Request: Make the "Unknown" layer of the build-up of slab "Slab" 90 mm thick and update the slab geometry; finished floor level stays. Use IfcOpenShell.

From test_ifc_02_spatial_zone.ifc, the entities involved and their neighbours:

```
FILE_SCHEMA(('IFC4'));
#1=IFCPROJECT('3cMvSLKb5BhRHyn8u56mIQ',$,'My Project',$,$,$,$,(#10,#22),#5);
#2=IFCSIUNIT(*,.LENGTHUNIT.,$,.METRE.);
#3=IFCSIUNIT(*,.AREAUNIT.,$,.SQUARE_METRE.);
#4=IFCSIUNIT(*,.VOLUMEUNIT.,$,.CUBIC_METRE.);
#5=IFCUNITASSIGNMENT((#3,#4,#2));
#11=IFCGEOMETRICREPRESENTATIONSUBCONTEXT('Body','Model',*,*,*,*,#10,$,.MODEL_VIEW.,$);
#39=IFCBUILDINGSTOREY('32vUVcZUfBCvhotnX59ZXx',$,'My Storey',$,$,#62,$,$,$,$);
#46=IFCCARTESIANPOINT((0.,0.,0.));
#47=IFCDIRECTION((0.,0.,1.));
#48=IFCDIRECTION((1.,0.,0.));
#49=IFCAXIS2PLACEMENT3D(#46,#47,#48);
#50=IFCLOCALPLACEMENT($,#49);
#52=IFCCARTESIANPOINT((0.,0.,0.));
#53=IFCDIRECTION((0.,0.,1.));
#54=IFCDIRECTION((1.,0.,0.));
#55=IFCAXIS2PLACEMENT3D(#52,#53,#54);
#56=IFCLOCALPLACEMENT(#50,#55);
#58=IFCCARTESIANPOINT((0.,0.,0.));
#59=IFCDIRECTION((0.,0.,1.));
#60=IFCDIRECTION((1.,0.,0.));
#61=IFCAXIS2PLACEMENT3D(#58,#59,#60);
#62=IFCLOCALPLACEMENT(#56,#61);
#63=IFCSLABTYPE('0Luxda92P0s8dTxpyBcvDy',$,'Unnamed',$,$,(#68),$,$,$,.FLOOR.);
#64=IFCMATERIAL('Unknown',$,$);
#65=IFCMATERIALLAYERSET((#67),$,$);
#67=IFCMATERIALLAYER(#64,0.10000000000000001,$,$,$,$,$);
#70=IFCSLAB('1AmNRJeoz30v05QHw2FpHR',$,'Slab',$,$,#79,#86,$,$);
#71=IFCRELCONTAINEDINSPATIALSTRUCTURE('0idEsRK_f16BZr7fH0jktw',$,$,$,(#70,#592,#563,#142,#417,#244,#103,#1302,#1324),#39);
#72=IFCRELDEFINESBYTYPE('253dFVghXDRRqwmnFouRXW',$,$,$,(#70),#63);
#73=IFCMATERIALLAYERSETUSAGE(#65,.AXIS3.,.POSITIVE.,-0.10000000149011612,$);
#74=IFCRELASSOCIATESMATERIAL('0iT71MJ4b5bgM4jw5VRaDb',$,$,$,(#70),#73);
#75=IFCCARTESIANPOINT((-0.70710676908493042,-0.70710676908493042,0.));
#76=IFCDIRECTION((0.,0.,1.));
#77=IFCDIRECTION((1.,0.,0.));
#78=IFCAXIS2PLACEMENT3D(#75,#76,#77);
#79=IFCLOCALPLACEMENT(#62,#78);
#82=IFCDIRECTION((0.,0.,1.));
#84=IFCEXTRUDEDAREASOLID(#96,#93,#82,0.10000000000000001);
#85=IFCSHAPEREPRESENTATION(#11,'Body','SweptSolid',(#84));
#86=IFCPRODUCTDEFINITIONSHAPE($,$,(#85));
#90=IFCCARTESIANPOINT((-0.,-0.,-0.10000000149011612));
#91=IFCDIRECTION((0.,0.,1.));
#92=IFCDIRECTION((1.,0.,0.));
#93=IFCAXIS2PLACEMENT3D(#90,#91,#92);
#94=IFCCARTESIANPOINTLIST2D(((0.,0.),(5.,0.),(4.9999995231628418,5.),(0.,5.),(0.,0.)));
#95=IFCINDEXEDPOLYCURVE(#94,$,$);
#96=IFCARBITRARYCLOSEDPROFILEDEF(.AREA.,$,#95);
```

```python
import ifcopenshell
import ifcopenshell.util.element
import ifcopenshell.util.representation
import ifcopenshell.util.unit

model = ifcopenshell.open("test_ifc_02_spatial_zone.ifc")
unit_scale = ifcopenshell.util.unit.calculate_unit_scale(model)

layer_set = model.by_id(65)
layer = next(l for l in layer_set.MaterialLayers if l.Material and l.Material.Name == "Unknown")
change = 0.09 / unit_scale - layer.LayerThickness
layer.LayerThickness += change

# Geometry does not follow the layer set by itself.
slabs = [e for e in ifcopenshell.util.element.get_elements_by_material(model, layer_set) if e.is_a("IfcSlab")]
for slab in sorted(slabs, key=lambda e: e.id()):
    body = ifcopenshell.util.representation.get_representation(slab, "Model", "Body")
    solid = body.Items[0]
    old_depth = solid.Depth
    solid.Depth += change
    # Extruded upwards: lower the start of the extrusion so the top stays.
    x, y, z = solid.Position.Location.Coordinates
    solid.Position.Location = model.createIfcCartesianPoint((x, y, z - change))
    print(slab.id(), f"{old_depth:g} -> {solid.Depth:g}")

# The layers are counted up from the underside, which has moved.
for usage in {ifcopenshell.util.element.get_material(slab) for slab in slabs}:
    usage.OffsetFromReferenceLine -= change

model.write("test_ifc_02_spatial_zone_v2.ifc")
```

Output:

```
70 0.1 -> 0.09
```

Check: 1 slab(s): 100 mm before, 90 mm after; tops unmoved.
